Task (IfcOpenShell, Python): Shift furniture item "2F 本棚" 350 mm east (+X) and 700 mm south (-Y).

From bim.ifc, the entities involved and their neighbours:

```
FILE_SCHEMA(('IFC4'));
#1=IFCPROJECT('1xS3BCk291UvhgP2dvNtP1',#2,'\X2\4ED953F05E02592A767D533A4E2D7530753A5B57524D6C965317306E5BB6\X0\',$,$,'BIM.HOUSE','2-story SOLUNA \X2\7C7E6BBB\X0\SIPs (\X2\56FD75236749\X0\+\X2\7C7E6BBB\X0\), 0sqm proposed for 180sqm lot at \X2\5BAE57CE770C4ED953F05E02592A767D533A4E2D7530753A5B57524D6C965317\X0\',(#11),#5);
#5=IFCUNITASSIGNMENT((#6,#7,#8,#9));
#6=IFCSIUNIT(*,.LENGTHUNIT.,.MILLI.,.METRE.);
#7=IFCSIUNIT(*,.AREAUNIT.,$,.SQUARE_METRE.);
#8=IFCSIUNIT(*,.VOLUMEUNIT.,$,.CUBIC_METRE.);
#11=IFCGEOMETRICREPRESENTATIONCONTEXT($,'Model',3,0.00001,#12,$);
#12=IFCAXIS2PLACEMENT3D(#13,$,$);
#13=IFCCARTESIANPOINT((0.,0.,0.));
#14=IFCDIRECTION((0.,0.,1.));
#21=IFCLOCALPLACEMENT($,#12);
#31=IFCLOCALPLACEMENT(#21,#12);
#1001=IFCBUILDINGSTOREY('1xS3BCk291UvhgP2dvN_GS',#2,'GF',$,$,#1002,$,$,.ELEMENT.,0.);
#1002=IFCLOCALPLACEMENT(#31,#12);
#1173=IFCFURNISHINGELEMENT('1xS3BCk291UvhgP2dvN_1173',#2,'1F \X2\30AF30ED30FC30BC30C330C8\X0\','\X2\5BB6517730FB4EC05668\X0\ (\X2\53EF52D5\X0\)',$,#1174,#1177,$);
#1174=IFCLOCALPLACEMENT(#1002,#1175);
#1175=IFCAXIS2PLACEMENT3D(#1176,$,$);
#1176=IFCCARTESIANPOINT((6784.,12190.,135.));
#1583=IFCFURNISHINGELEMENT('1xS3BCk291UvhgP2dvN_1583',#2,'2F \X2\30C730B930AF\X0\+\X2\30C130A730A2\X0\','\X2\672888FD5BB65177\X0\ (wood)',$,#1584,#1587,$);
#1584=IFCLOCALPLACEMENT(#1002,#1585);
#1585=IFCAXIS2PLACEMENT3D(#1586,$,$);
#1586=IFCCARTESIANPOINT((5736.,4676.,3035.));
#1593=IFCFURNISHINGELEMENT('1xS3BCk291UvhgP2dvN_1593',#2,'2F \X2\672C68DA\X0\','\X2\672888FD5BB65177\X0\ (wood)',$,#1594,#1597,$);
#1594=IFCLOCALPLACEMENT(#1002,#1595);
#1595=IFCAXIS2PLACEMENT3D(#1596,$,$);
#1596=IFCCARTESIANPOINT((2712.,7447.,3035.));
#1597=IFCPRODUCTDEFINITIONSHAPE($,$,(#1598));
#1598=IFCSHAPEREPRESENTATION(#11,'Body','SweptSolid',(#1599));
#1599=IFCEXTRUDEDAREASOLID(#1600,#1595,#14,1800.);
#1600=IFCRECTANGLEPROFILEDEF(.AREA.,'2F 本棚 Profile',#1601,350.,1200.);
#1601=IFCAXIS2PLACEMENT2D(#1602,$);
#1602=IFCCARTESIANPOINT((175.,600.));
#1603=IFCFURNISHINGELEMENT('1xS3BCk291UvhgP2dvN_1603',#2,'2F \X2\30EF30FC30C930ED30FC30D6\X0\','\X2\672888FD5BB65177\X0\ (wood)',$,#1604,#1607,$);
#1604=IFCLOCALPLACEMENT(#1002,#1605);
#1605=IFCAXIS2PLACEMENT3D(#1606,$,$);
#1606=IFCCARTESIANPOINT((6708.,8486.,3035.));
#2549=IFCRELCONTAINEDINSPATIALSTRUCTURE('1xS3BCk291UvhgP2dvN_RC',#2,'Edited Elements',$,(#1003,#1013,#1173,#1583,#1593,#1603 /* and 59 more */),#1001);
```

```python
import ifcopenshell
import ifcopenshell.api.geometry
import ifcopenshell.util.placement
import ifcopenshell.util.unit

model = ifcopenshell.open("bim.ifc")
unit_scale = ifcopenshell.util.unit.calculate_unit_scale(model)

item = model.by_guid("1xS3BCk291UvhgP2dvN_1593")
matrix = ifcopenshell.util.placement.get_local_placement(item.ObjectPlacement)
matrix[0, 3] += 0.35 / unit_scale
matrix[1, 3] -= 0.7 / unit_scale
ifcopenshell.api.geometry.edit_object_placement(model, product=item, matrix=matrix, is_si=False)

print(ifcopenshell.util.placement.get_local_placement(item.ObjectPlacement).round(3) + 0.0)

model.write("bim_rev.ifc")
```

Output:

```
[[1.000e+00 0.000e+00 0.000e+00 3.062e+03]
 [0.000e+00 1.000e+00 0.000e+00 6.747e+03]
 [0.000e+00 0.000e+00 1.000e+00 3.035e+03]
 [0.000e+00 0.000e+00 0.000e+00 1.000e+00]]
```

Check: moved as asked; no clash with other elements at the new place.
